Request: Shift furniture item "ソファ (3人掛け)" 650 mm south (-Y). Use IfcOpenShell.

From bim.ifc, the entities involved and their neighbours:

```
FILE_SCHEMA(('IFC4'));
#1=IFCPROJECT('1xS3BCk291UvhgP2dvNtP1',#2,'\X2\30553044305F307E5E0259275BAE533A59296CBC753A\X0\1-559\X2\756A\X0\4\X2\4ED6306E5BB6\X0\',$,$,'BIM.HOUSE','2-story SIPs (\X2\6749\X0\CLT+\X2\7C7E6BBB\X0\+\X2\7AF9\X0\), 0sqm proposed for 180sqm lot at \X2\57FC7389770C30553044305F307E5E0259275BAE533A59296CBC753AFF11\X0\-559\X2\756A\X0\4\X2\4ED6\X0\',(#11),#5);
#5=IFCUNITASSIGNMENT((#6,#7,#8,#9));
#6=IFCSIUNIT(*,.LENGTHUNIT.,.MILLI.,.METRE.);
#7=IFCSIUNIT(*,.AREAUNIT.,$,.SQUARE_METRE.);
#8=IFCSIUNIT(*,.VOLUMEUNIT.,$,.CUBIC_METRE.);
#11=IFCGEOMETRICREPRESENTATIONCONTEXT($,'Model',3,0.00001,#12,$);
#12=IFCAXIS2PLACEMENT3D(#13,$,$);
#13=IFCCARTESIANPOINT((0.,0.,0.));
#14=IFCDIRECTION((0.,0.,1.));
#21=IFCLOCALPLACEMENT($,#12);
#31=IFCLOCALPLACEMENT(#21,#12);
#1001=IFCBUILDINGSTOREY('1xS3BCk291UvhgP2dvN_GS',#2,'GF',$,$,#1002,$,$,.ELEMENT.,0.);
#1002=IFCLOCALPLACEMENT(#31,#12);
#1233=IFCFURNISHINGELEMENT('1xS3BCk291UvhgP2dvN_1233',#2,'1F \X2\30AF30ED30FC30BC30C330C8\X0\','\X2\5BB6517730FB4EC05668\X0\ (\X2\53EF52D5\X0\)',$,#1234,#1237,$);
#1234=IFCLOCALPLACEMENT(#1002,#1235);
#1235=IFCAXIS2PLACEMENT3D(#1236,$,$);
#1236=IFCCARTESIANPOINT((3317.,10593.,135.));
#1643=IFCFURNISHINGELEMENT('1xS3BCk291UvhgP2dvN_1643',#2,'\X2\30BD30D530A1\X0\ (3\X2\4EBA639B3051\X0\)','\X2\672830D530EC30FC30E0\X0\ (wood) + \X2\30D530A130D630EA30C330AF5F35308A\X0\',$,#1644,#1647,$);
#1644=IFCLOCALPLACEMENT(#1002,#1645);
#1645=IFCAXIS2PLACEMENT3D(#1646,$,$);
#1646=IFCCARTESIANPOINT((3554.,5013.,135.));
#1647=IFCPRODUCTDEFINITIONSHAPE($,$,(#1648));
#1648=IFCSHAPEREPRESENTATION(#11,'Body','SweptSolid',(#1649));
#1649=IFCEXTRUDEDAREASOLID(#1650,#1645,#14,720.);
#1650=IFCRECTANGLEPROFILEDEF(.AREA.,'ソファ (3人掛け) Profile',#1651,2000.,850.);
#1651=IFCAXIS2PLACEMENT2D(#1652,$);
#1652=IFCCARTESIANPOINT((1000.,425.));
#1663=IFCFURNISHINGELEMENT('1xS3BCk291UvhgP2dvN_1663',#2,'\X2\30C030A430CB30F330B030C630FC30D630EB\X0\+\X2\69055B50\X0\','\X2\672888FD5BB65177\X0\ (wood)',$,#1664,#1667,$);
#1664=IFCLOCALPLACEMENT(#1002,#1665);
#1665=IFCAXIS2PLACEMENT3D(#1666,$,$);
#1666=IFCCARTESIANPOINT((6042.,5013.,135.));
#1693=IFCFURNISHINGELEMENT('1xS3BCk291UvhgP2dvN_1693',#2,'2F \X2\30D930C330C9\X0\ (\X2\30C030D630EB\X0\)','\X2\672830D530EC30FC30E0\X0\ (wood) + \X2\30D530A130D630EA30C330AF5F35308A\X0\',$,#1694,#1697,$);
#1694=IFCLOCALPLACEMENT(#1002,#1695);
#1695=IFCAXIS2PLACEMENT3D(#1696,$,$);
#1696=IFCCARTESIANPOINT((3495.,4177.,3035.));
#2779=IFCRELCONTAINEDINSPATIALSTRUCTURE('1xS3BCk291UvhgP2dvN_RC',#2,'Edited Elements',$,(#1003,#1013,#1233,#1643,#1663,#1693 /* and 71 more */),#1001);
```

```python
import ifcopenshell
import ifcopenshell.api.geometry
import ifcopenshell.util.placement
import ifcopenshell.util.unit

model = ifcopenshell.open("bim.ifc")
unit_scale = ifcopenshell.util.unit.calculate_unit_scale(model)

item = model.by_guid("1xS3BCk291UvhgP2dvN_1643")
matrix = ifcopenshell.util.placement.get_local_placement(item.ObjectPlacement)
matrix[1, 3] -= 0.65 / unit_scale
ifcopenshell.api.geometry.edit_object_placement(model, product=item, matrix=matrix, is_si=False)

print(ifcopenshell.util.placement.get_local_placement(item.ObjectPlacement).round(3) + 0.0)

model.write("bim_updated.ifc")
```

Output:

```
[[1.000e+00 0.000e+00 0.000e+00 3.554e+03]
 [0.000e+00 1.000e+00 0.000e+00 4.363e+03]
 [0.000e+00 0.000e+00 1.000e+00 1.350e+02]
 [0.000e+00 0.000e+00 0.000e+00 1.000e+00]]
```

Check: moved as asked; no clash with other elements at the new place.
